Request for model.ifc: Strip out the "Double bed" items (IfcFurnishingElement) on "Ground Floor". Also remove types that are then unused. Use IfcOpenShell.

First a look at what the model holds.

```python
import ifcopenshell
import ifcopenshell.util.element

model = ifcopenshell.open("model.ifc")
print(model.schema)
storey = next(s for s in model.by_type("IfcBuildingStorey") if s.Name == "Ground Floor")
furniture = [e for e in ifcopenshell.util.element.get_decomposition(storey) if e.is_a("IfcFurnishingElement")]
seen = {}
for e in furniture:
    element_type = ifcopenshell.util.element.get_type(e)
    name = element_type.Name if element_type not in (None, e) else None
    seen[name] = seen.get(name, 0) + 1
for name, count in sorted(seen.items(), key=str):
    print(count, "x", name)
```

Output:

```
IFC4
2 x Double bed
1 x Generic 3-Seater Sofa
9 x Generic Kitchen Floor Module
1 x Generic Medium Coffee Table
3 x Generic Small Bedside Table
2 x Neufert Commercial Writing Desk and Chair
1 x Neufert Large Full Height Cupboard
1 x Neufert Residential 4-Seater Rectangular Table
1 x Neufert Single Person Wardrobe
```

```python
import ifcopenshell
import ifcopenshell.api.root
import ifcopenshell.util.element

model = ifcopenshell.open("model.ifc")

storey = next(s for s in model.by_type("IfcBuildingStorey") if s.Name == "Ground Floor")
furniture = [e for e in ifcopenshell.util.element.get_decomposition(storey) if e.is_a("IfcFurnishingElement")]
targets = [e for e in furniture if (t := ifcopenshell.util.element.get_type(e)) not in (None, e) and t.Name == "Double bed"]
types = {ifcopenshell.util.element.get_type(e) for e in targets} - {None, *targets}

for e in targets:
    ifcopenshell.api.root.remove_product(model, product=e)
print(len(targets), "removed")

unused = [t for t in types if not ifcopenshell.util.element.get_types(t)]
for t in unused:
    ifcopenshell.api.root.remove_product(model, product=t)
print(len(unused), "unused types removed")

model.write("model_rev.ifc")
```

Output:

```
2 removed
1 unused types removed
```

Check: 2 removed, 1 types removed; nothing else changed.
